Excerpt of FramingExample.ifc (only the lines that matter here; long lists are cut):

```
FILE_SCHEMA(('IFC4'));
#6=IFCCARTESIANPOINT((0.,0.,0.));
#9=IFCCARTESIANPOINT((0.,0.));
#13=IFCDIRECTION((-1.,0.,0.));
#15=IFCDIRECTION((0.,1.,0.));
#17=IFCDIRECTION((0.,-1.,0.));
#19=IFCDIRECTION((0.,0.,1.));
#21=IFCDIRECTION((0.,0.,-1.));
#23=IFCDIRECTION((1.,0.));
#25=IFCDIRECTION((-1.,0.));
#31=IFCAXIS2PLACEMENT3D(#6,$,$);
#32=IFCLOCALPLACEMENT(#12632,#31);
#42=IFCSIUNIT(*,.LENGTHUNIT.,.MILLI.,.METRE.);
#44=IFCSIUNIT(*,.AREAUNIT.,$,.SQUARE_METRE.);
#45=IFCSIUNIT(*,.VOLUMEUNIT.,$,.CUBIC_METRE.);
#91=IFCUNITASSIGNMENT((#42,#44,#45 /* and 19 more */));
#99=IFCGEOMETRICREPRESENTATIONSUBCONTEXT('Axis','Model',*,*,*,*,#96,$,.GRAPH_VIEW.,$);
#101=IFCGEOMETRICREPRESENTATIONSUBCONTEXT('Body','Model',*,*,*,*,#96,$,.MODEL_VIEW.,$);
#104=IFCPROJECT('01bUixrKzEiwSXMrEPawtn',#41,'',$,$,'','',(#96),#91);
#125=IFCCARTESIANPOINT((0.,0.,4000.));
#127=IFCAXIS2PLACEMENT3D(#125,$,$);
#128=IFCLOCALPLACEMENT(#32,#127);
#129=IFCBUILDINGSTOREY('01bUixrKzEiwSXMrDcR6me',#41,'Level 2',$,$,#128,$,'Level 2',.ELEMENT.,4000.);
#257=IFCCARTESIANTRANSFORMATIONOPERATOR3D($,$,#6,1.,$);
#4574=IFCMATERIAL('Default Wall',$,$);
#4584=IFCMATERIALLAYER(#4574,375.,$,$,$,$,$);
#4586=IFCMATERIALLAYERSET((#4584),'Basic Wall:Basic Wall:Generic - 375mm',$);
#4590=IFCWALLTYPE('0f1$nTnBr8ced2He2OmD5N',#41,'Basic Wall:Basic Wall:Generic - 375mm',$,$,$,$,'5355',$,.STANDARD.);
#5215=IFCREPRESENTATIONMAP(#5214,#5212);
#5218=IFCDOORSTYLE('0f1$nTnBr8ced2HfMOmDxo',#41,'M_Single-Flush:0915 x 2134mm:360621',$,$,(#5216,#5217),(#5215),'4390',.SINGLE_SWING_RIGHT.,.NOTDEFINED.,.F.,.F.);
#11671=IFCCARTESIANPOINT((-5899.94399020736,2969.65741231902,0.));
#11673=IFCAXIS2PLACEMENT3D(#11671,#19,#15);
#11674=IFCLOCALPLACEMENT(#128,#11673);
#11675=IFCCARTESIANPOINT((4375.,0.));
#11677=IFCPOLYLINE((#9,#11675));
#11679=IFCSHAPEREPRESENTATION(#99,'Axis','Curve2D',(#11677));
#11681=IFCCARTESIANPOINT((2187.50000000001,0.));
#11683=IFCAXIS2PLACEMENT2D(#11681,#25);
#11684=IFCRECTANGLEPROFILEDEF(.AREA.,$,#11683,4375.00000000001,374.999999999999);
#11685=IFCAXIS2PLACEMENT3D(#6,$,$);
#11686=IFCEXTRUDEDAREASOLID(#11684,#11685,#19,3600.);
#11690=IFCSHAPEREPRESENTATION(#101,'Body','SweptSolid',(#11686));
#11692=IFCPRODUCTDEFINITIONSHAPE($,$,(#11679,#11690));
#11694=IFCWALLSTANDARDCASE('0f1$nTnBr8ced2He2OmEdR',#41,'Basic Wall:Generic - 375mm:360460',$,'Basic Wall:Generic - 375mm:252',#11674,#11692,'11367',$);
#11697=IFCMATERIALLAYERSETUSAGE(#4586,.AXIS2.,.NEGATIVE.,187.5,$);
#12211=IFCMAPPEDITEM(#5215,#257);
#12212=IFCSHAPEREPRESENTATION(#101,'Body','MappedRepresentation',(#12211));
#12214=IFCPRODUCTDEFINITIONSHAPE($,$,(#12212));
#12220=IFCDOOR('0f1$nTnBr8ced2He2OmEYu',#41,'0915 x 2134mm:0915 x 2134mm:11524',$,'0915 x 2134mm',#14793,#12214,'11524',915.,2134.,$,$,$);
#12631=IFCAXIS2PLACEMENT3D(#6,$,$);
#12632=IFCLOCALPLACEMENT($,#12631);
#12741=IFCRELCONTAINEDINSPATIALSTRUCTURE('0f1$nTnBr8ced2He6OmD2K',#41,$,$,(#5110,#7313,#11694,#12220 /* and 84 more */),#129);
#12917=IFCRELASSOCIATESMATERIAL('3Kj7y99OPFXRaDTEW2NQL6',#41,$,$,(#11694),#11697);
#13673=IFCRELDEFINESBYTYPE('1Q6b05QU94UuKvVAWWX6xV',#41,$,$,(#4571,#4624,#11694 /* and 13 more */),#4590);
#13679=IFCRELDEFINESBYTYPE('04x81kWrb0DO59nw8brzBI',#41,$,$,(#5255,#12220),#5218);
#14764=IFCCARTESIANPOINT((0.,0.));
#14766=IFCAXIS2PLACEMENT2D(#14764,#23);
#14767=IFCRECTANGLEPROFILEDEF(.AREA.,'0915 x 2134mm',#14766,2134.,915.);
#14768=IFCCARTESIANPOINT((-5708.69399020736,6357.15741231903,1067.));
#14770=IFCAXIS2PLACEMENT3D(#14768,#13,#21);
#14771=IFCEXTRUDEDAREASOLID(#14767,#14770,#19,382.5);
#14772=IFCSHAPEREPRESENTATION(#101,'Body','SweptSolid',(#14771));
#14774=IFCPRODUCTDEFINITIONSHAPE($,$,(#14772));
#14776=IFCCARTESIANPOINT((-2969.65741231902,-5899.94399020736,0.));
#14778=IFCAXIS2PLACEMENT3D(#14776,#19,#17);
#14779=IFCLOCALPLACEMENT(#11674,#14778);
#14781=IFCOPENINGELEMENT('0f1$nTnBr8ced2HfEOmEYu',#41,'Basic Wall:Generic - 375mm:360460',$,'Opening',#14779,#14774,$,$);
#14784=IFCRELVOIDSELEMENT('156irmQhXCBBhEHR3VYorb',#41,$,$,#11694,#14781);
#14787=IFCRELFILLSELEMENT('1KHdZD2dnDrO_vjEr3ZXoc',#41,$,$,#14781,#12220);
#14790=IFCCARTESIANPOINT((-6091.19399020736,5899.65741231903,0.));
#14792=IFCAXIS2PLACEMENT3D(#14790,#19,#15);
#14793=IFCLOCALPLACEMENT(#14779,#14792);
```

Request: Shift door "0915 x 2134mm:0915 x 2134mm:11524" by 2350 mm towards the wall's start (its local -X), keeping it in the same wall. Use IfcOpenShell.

```python
import ifcopenshell
import ifcopenshell.api.geometry
import ifcopenshell.util.placement
import ifcopenshell.util.unit

model = ifcopenshell.open("FramingExample.ifc")
unit_scale = ifcopenshell.util.unit.calculate_unit_scale(model)

door = model.by_id(12220)
opening = door.FillsVoids[0].RelatingOpeningElement
wall = opening.VoidsElements[0].RelatingBuildingElement

wall_matrix = ifcopenshell.util.placement.get_local_placement(wall.ObjectPlacement)
shift = wall_matrix[:3, 0] * -2.35 / unit_scale
before = ifcopenshell.util.placement.get_local_placement(door.ObjectPlacement)[:3, 3].copy()

# The door is placed relative to its opening, so it follows when the opening moves.
matrix = ifcopenshell.util.placement.get_local_placement(opening.ObjectPlacement)
matrix[:3, 3] += shift
ifcopenshell.api.geometry.edit_object_placement(
    model, product=opening, matrix=matrix, is_si=False, should_transform_children=True
)

after = ifcopenshell.util.placement.get_local_placement(door.ObjectPlacement)[:3, 3]
print("door moved by", (after - before).round(3) + 0.0)

model.write("FramingExample_updated.ifc")
```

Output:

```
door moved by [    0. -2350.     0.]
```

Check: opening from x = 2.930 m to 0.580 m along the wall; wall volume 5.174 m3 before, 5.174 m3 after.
